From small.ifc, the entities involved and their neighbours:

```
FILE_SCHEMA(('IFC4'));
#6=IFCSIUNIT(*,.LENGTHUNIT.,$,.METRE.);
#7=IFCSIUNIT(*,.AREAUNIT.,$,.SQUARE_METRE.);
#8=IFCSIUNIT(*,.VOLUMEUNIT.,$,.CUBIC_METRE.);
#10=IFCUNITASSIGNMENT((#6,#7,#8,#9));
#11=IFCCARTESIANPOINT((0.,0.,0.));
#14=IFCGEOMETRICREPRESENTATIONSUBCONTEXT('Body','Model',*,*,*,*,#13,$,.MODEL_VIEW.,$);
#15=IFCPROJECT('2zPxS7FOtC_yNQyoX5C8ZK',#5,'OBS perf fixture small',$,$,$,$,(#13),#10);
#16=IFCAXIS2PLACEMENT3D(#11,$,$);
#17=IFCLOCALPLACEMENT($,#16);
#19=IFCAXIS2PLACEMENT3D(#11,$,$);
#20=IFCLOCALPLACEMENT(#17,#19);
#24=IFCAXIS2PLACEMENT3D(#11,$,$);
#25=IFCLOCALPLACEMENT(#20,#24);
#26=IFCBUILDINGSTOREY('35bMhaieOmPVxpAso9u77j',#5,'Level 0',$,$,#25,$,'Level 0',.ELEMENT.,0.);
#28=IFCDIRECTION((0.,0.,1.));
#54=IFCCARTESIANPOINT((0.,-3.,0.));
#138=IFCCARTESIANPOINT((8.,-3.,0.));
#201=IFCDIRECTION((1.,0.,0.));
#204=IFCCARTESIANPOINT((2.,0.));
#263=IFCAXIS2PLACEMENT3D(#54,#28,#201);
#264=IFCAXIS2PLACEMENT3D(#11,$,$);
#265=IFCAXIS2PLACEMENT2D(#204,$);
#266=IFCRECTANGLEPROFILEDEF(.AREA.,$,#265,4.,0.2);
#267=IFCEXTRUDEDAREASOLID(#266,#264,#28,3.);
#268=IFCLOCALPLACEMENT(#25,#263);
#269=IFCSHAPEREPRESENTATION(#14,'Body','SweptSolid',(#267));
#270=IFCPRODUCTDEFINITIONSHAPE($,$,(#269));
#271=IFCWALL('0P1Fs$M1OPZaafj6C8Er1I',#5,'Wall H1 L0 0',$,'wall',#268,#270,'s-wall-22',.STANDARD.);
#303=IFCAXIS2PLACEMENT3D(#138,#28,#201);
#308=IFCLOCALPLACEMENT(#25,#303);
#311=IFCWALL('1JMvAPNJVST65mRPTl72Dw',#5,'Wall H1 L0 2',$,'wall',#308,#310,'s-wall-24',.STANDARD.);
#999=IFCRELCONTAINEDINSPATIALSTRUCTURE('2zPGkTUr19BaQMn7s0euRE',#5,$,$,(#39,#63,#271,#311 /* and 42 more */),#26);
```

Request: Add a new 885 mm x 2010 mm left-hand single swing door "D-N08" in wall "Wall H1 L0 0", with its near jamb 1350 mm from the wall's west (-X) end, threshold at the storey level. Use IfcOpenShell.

```python
import numpy as np
import ifcopenshell
import ifcopenshell.api.feature
import ifcopenshell.api.geometry
import ifcopenshell.api.root
import ifcopenshell.api.spatial
import ifcopenshell.geom
import ifcopenshell.util.element
import ifcopenshell.util.placement
import ifcopenshell.util.representation
import ifcopenshell.util.shape
import ifcopenshell.util.unit

model = ifcopenshell.open("small.ifc")
unit_scale = ifcopenshell.util.unit.calculate_unit_scale(model)
settings = ifcopenshell.geom.settings()


def volume(element):
    """Net volume in cubic metres, openings subtracted."""
    shape = ifcopenshell.geom.create_shape(settings, element)
    return ifcopenshell.util.shape.get_volume(shape.geometry)


wall = model.by_guid("0P1Fs$M1OPZaafj6C8Er1I")
storey = ifcopenshell.util.element.get_container(wall, ifc_class="IfcBuildingStorey")
context = ifcopenshell.util.representation.get_context(model, "Model", "Body", "MODEL_VIEW")
before = volume(wall)

width, height, from_end, sill = 0.885, 2.01, 1.35, 0.0  # metres

# The wall runs along its own X axis, and the end named is its -X end.
wall_shape = ifcopenshell.geom.create_shape(settings, wall)
x, y, z = ifcopenshell.util.shape.get_vertices(wall_shape.geometry).T
start = x.min() + from_end
face, thickness = float(y.min()), float(y.max() - y.min())
wall_matrix = ifcopenshell.util.placement.get_local_placement(wall.ObjectPlacement)
level = ifcopenshell.util.placement.get_local_placement(storey.ObjectPlacement)[2, 3]


def in_wall(x, y):
    """Placement at x, y metres in the wall's axes, at sill height."""
    matrix = wall_matrix.copy()
    matrix[:, 3] = wall_matrix @ np.array([x / unit_scale, y / unit_scale, 0.0, 1.0])
    matrix[2, 3] = level + sill / unit_scale
    return matrix


# Opening: a box that overshoots both wall faces by 50 mm.
opening = ifcopenshell.api.root.create_entity(model, ifc_class="IfcOpeningElement", predefined_type="OPENING")
box = ifcopenshell.api.geometry.add_wall_representation(
    model, context=context, length=width, height=height, thickness=thickness + 0.1
)
ifcopenshell.api.geometry.assign_representation(model, product=opening, representation=box)
ifcopenshell.api.geometry.edit_object_placement(model, product=opening, matrix=in_wall(start, face - 0.05), is_si=False)
ifcopenshell.api.feature.add_feature(model, feature=opening, element=wall)

door = ifcopenshell.api.root.create_entity(model, ifc_class="IfcDoor", name="D-N08", predefined_type="DOOR")
door.OverallWidth, door.OverallHeight = width / unit_scale, height / unit_scale
door.OperationType = "SINGLE_SWING_LEFT"
body = ifcopenshell.api.geometry.add_door_representation(
    model,
    context=context,
    overall_width=door.OverallWidth,
    overall_height=door.OverallHeight,
    operation_type="SINGLE_SWING_LEFT",
    lining_properties={"LiningDepth": thickness / unit_scale, "ThresholdDepth": thickness / unit_scale},
)
ifcopenshell.api.geometry.assign_representation(model, product=door, representation=body)
ifcopenshell.api.spatial.assign_container(model, products=[door], relating_structure=storey)
ifcopenshell.api.feature.add_filling(model, opening=opening, element=door)

# The lining spans the wall, so the door starts at the wall face.
ifcopenshell.api.geometry.edit_object_placement(model, product=door, matrix=in_wall(start, face), is_si=False)

after = volume(wall)

print(f"wall volume {before:.3f} -> {after:.3f} m3")

model.write("small_rev.ifc")
```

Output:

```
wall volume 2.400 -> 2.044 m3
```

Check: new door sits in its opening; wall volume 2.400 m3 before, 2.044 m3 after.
